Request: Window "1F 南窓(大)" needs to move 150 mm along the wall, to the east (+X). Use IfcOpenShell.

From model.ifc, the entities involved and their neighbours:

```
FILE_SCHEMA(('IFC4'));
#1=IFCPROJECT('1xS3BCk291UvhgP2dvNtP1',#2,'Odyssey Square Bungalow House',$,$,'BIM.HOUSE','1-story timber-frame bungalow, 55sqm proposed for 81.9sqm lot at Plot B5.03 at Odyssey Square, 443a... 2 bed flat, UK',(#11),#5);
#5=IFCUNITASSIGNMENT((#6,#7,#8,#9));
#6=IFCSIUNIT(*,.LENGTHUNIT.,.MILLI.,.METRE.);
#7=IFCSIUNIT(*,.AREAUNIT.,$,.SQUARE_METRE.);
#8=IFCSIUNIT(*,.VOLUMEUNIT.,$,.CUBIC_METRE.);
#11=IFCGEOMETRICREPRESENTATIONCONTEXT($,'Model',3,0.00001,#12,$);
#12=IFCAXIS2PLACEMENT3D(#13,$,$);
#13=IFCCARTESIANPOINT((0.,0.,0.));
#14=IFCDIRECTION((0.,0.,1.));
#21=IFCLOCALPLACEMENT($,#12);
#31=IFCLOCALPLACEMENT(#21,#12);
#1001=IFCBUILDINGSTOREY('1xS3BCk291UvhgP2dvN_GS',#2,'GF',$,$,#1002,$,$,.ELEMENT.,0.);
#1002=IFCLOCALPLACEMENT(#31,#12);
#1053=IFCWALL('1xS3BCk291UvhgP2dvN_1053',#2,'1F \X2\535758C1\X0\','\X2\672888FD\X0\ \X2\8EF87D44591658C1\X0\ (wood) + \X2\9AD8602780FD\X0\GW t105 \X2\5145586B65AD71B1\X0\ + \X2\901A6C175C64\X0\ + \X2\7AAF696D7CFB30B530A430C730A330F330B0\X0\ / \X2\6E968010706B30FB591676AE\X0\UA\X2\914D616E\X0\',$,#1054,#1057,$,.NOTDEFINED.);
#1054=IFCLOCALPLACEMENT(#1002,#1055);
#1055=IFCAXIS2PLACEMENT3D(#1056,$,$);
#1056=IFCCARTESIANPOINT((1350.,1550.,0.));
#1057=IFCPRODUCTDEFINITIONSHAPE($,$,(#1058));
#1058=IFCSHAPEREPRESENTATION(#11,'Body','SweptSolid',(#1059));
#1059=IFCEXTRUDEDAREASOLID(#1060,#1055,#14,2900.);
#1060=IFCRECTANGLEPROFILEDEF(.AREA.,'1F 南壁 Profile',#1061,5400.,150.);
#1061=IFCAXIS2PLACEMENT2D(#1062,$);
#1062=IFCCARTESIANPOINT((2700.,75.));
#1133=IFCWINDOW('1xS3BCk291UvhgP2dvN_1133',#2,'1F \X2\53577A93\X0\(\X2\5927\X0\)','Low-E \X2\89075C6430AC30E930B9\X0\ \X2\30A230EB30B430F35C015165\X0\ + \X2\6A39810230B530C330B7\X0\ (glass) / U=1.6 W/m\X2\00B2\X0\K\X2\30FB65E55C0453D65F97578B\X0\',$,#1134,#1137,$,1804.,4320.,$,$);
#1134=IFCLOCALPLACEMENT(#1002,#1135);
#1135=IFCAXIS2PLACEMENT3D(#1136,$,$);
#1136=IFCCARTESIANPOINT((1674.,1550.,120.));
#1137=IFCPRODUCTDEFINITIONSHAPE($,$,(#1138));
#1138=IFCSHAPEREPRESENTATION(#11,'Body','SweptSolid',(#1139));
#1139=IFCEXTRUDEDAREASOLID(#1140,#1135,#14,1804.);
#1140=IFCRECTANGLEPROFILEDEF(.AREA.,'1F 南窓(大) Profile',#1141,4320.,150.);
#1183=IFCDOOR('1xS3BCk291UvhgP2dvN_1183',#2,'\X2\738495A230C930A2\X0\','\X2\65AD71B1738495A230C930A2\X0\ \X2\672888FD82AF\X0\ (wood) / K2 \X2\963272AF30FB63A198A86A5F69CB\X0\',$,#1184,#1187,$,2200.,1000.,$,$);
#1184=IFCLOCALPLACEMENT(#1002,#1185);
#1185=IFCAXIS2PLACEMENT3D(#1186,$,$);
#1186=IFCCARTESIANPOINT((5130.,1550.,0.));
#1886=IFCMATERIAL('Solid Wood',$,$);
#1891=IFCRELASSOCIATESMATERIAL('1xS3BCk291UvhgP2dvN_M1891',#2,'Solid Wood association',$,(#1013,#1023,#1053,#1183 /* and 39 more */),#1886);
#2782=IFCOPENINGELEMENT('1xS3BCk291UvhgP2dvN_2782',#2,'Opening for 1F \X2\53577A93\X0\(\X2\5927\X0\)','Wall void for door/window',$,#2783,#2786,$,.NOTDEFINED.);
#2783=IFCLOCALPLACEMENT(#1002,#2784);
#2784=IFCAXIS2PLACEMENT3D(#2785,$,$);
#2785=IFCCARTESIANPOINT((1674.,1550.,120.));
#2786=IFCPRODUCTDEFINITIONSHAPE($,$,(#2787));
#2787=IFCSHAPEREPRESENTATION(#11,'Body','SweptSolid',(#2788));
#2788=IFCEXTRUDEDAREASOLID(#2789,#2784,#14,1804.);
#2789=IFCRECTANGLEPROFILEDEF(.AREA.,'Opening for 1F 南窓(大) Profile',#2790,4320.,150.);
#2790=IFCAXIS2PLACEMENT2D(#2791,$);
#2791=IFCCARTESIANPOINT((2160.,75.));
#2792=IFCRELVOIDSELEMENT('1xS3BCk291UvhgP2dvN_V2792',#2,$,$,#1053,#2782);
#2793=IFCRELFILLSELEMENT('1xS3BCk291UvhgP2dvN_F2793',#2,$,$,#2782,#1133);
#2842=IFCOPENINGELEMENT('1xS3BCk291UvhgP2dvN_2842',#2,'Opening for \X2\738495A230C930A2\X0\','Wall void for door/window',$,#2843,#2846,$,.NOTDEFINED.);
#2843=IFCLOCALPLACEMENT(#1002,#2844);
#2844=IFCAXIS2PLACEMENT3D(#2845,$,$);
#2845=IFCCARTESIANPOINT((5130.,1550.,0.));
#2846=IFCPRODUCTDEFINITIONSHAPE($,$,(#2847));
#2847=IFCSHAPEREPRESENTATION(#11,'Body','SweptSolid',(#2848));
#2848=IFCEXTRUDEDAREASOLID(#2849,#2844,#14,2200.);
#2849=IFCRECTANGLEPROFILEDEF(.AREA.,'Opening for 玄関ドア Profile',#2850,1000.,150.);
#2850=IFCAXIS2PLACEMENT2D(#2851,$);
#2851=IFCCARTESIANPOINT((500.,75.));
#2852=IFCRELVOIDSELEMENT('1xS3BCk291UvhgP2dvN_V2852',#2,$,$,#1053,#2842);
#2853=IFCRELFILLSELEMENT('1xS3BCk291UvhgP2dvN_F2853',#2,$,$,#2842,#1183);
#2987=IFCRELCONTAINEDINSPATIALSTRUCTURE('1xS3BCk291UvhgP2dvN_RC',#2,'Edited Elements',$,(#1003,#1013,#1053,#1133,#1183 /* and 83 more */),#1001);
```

```python
import ifcopenshell
import ifcopenshell.api.geometry
import ifcopenshell.util.placement
import ifcopenshell.util.unit

model = ifcopenshell.open("model.ifc")
unit_scale = ifcopenshell.util.unit.calculate_unit_scale(model)

window = model.by_guid("1xS3BCk291UvhgP2dvN_1133")
opening = window.FillsVoids[0].RelatingOpeningElement
wall = opening.VoidsElements[0].RelatingBuildingElement

wall_matrix = ifcopenshell.util.placement.get_local_placement(wall.ObjectPlacement)
shift = wall_matrix[:3, 0] * 0.15 / unit_scale
before = ifcopenshell.util.placement.get_local_placement(window.ObjectPlacement)[:3, 3].copy()

# The window is not placed relative to its opening, so move both.
for product in (opening, window):
    matrix = ifcopenshell.util.placement.get_local_placement(product.ObjectPlacement)
    matrix[:3, 3] += shift
    ifcopenshell.api.geometry.edit_object_placement(model, product=product, matrix=matrix, is_si=False)

after = ifcopenshell.util.placement.get_local_placement(window.ObjectPlacement)[:3, 3]
print("window moved by", (after - before).round(3) + 0.0)

model.write("model-out.ifc")
```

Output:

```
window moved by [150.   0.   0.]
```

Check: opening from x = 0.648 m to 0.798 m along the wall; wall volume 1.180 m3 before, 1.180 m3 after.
